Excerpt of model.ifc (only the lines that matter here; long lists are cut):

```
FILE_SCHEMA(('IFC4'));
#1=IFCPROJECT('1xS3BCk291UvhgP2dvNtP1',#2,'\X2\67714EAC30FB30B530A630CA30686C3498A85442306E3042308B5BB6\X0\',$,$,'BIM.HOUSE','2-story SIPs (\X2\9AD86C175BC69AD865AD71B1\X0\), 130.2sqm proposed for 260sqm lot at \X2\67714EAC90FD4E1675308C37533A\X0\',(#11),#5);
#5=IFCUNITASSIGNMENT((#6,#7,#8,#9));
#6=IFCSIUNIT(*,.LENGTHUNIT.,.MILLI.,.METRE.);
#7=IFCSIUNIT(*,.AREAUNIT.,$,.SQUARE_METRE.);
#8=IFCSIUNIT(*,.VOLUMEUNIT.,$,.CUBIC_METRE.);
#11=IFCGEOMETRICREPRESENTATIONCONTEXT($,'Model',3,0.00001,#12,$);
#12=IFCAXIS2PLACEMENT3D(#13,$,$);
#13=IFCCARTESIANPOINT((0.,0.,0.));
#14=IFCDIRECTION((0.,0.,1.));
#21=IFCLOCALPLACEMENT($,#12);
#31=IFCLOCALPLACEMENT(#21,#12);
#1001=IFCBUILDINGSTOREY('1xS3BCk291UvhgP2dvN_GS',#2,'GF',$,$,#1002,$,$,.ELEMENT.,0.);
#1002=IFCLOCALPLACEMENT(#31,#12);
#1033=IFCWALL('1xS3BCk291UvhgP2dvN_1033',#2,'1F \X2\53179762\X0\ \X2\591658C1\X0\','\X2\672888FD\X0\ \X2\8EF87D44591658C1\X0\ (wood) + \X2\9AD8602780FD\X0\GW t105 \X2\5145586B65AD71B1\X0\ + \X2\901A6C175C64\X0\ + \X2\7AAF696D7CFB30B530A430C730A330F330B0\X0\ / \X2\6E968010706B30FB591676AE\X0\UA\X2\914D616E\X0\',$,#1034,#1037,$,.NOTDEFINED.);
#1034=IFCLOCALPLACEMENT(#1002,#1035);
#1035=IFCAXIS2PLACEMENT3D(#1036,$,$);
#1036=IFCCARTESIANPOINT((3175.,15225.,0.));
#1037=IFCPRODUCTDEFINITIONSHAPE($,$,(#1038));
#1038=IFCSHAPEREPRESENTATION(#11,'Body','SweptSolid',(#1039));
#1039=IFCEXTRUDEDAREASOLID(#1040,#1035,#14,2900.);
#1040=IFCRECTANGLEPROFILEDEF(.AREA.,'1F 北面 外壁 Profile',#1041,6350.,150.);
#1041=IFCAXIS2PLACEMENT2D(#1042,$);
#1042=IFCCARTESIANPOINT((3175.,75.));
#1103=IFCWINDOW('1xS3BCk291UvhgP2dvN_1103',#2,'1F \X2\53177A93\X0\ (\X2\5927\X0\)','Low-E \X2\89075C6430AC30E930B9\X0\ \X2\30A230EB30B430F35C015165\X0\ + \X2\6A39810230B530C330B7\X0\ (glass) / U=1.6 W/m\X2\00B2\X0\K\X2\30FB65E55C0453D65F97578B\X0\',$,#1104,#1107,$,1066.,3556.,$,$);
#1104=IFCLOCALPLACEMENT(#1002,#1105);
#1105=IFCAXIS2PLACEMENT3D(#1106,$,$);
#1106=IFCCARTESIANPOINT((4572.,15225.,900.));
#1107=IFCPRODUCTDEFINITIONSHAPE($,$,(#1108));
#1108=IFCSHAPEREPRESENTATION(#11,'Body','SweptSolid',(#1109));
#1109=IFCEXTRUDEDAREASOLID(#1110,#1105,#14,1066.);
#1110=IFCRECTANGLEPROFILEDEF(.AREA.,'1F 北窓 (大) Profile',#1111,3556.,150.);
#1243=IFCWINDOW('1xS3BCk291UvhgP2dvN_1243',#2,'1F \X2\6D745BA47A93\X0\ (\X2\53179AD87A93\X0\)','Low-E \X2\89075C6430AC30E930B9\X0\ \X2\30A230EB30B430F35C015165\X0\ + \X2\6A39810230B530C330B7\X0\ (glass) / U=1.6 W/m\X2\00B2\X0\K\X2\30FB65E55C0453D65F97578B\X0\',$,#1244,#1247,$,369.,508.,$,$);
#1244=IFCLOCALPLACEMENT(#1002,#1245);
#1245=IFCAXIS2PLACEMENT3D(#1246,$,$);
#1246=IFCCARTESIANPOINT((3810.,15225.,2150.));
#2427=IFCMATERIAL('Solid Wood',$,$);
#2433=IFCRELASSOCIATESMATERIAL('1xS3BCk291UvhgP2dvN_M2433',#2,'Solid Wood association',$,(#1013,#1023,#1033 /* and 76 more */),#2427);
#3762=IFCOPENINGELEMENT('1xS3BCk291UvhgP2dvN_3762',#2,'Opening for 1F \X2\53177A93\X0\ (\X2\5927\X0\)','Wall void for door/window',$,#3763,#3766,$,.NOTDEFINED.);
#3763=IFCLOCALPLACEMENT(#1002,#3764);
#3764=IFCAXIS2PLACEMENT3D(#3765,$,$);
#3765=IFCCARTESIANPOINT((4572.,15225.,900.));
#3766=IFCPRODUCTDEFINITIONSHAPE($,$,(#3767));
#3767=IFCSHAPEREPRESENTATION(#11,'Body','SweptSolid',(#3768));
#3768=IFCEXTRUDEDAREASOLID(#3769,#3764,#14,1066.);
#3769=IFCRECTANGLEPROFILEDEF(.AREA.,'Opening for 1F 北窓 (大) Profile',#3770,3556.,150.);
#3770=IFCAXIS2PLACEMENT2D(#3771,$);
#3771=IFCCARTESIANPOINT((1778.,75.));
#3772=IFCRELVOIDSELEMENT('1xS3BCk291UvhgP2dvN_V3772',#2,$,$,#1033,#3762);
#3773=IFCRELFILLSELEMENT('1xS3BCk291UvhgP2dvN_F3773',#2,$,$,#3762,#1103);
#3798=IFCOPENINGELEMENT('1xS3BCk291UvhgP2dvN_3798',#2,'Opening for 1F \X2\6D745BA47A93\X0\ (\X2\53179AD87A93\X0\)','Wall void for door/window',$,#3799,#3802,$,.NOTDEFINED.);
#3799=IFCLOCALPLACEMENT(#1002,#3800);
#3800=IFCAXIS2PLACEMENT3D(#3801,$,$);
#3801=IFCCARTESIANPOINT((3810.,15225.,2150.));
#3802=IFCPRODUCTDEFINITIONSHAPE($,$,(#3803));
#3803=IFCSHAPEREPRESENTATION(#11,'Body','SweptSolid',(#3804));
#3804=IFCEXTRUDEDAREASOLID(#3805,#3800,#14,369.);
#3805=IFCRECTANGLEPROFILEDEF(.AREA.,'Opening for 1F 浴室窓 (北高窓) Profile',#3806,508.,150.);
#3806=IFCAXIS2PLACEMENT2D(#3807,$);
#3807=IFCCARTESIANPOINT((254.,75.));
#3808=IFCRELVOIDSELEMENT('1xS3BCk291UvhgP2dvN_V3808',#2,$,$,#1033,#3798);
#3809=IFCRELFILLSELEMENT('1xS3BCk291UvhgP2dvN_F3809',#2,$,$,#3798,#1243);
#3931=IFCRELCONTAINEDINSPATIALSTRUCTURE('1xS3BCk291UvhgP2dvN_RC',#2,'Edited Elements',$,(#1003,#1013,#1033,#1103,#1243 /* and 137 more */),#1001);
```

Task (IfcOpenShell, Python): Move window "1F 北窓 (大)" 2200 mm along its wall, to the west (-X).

```python
import ifcopenshell
import ifcopenshell.api.geometry
import ifcopenshell.util.placement
import ifcopenshell.util.unit

model = ifcopenshell.open("model.ifc")
unit_scale = ifcopenshell.util.unit.calculate_unit_scale(model)

window = model.by_guid("1xS3BCk291UvhgP2dvN_1103")
opening = window.FillsVoids[0].RelatingOpeningElement
wall = opening.VoidsElements[0].RelatingBuildingElement

wall_matrix = ifcopenshell.util.placement.get_local_placement(wall.ObjectPlacement)
shift = wall_matrix[:3, 0] * -2.2 / unit_scale
before = ifcopenshell.util.placement.get_local_placement(window.ObjectPlacement)[:3, 3].copy()

# The window is not placed relative to its opening, so move both.
for product in (opening, window):
    matrix = ifcopenshell.util.placement.get_local_placement(product.ObjectPlacement)
    matrix[:3, 3] += shift
    ifcopenshell.api.geometry.edit_object_placement(model, product=product, matrix=matrix, is_si=False)

after = ifcopenshell.util.placement.get_local_placement(window.ObjectPlacement)[:3, 3]
print("window moved by", (after - before).round(3) + 0.0)

model.write("model_edited.ifc")
```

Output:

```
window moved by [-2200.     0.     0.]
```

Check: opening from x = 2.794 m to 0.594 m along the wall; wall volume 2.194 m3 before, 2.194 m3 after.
